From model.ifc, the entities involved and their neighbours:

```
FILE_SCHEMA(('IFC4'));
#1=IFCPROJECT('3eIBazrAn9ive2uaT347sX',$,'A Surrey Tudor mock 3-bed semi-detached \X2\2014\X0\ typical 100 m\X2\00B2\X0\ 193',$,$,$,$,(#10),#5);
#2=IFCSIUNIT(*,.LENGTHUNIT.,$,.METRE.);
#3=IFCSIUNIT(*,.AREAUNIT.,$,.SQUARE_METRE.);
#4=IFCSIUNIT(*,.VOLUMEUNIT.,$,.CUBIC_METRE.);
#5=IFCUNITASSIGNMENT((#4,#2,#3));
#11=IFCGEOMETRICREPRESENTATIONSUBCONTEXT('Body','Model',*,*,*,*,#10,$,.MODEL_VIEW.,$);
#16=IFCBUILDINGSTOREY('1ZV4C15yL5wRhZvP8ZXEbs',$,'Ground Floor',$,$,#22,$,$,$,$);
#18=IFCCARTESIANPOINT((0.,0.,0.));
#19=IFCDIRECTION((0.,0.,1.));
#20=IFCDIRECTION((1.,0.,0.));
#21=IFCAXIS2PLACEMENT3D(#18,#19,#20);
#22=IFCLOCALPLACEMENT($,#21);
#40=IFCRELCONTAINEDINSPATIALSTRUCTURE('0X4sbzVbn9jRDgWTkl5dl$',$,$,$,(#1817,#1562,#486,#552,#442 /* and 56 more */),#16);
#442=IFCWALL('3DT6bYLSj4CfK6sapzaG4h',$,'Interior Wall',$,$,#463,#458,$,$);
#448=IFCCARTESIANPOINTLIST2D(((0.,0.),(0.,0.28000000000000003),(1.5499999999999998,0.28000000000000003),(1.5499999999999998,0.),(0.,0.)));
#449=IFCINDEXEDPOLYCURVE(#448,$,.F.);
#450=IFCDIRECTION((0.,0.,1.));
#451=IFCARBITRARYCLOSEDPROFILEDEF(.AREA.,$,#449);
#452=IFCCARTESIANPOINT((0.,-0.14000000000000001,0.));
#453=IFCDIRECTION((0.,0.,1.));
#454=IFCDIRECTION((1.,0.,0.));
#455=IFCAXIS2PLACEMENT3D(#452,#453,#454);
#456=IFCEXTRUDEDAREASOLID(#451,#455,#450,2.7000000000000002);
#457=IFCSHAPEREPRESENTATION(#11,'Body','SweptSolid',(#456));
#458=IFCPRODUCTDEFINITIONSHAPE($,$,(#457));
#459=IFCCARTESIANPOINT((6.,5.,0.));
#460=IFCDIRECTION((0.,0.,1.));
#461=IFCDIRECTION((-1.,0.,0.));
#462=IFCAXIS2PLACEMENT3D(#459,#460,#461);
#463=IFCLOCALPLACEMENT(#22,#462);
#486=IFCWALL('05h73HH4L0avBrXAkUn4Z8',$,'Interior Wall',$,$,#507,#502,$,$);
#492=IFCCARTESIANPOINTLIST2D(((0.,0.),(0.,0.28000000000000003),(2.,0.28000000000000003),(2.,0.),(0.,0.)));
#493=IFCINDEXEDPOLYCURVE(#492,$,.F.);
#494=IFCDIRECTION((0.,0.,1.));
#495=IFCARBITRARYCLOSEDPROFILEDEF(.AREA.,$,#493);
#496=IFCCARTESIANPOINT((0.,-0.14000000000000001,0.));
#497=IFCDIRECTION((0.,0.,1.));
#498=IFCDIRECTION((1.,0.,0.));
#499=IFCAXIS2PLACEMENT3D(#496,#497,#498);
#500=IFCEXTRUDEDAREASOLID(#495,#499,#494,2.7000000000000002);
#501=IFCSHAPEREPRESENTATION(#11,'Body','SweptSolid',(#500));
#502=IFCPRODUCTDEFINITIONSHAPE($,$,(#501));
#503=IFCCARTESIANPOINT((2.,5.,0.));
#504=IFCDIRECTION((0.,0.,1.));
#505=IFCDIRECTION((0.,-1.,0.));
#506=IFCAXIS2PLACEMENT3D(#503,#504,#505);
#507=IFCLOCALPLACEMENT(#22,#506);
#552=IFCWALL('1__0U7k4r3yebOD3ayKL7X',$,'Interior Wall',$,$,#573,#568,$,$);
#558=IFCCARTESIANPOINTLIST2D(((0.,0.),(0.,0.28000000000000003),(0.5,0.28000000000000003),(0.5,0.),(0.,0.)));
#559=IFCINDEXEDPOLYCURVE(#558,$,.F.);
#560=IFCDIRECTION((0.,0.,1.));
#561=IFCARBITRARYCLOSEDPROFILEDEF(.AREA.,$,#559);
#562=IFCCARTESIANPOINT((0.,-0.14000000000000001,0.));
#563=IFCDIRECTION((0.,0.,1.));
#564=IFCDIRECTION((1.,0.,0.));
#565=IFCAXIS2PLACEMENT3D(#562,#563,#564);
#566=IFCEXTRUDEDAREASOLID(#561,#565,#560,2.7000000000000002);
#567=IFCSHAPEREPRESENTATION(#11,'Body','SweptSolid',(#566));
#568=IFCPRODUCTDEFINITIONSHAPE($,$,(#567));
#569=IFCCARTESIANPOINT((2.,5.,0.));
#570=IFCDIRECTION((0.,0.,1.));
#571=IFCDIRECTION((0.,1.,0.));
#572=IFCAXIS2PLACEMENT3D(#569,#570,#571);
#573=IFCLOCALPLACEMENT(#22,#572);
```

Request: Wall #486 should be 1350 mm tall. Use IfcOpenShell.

```python
import ifcopenshell
import ifcopenshell.geom
import ifcopenshell.util.representation
import ifcopenshell.util.shape
import ifcopenshell.util.unit

model = ifcopenshell.open("model.ifc")
unit_scale = ifcopenshell.util.unit.calculate_unit_scale(model)
settings = ifcopenshell.geom.settings()


def volume(element):
    """Net volume in cubic metres, openings subtracted."""
    shape = ifcopenshell.geom.create_shape(settings, element)
    return ifcopenshell.util.shape.get_volume(shape.geometry)


wall = model.by_id(486)
before = volume(wall)

body = ifcopenshell.util.representation.get_representation(wall, "Model", "Body")
solid = body.Items[0]
old_height = solid.Depth
solid.Depth = 1.35 / unit_scale
after = volume(wall)

print(f"height {old_height:g} -> {solid.Depth:g}, volume {before:.3f} -> {after:.3f} m3")

model.write("model_edited.ifc")
```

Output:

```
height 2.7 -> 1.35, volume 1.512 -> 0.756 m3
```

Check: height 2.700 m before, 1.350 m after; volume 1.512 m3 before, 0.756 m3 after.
